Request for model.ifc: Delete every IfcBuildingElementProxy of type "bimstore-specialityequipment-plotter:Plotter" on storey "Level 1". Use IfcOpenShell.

First a look at what the model holds.

```python
import ifcopenshell
import ifcopenshell.util.element

model = ifcopenshell.open("model.ifc")
print(model.schema)
storey = next(s for s in model.by_type("IfcBuildingStorey") if s.Name == "Level 1")
proxies = [e for e in ifcopenshell.util.element.get_decomposition(storey) if e.is_a("IfcBuildingElementProxy")]
seen = {}
for e in proxies:
    element_type = ifcopenshell.util.element.get_type(e)
    name = element_type.Name if element_type not in (None, e) else None
    seen[name] = seen.get(name, 0) + 1
for name, count in sorted(seen.items(), key=str):
    print(count, "x", name)
```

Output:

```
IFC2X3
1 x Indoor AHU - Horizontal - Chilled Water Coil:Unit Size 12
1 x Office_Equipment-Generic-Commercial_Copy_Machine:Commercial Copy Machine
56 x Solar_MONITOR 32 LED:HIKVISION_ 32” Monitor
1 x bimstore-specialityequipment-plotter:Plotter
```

```python
import ifcopenshell
import ifcopenshell.api.root
import ifcopenshell.util.element

model = ifcopenshell.open("model.ifc")

storey = next(s for s in model.by_type("IfcBuildingStorey") if s.Name == "Level 1")
proxies = [e for e in ifcopenshell.util.element.get_decomposition(storey) if e.is_a("IfcBuildingElementProxy")]
targets = [e for e in proxies if (t := ifcopenshell.util.element.get_type(e)) not in (None, e) and t.Name == "bimstore-specialityequipment-plotter:Plotter"]

for e in targets:
    ifcopenshell.api.root.remove_product(model, product=e)
print(len(targets), "removed")

model.write("model_edited.ifc")
```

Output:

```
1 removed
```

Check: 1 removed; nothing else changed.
